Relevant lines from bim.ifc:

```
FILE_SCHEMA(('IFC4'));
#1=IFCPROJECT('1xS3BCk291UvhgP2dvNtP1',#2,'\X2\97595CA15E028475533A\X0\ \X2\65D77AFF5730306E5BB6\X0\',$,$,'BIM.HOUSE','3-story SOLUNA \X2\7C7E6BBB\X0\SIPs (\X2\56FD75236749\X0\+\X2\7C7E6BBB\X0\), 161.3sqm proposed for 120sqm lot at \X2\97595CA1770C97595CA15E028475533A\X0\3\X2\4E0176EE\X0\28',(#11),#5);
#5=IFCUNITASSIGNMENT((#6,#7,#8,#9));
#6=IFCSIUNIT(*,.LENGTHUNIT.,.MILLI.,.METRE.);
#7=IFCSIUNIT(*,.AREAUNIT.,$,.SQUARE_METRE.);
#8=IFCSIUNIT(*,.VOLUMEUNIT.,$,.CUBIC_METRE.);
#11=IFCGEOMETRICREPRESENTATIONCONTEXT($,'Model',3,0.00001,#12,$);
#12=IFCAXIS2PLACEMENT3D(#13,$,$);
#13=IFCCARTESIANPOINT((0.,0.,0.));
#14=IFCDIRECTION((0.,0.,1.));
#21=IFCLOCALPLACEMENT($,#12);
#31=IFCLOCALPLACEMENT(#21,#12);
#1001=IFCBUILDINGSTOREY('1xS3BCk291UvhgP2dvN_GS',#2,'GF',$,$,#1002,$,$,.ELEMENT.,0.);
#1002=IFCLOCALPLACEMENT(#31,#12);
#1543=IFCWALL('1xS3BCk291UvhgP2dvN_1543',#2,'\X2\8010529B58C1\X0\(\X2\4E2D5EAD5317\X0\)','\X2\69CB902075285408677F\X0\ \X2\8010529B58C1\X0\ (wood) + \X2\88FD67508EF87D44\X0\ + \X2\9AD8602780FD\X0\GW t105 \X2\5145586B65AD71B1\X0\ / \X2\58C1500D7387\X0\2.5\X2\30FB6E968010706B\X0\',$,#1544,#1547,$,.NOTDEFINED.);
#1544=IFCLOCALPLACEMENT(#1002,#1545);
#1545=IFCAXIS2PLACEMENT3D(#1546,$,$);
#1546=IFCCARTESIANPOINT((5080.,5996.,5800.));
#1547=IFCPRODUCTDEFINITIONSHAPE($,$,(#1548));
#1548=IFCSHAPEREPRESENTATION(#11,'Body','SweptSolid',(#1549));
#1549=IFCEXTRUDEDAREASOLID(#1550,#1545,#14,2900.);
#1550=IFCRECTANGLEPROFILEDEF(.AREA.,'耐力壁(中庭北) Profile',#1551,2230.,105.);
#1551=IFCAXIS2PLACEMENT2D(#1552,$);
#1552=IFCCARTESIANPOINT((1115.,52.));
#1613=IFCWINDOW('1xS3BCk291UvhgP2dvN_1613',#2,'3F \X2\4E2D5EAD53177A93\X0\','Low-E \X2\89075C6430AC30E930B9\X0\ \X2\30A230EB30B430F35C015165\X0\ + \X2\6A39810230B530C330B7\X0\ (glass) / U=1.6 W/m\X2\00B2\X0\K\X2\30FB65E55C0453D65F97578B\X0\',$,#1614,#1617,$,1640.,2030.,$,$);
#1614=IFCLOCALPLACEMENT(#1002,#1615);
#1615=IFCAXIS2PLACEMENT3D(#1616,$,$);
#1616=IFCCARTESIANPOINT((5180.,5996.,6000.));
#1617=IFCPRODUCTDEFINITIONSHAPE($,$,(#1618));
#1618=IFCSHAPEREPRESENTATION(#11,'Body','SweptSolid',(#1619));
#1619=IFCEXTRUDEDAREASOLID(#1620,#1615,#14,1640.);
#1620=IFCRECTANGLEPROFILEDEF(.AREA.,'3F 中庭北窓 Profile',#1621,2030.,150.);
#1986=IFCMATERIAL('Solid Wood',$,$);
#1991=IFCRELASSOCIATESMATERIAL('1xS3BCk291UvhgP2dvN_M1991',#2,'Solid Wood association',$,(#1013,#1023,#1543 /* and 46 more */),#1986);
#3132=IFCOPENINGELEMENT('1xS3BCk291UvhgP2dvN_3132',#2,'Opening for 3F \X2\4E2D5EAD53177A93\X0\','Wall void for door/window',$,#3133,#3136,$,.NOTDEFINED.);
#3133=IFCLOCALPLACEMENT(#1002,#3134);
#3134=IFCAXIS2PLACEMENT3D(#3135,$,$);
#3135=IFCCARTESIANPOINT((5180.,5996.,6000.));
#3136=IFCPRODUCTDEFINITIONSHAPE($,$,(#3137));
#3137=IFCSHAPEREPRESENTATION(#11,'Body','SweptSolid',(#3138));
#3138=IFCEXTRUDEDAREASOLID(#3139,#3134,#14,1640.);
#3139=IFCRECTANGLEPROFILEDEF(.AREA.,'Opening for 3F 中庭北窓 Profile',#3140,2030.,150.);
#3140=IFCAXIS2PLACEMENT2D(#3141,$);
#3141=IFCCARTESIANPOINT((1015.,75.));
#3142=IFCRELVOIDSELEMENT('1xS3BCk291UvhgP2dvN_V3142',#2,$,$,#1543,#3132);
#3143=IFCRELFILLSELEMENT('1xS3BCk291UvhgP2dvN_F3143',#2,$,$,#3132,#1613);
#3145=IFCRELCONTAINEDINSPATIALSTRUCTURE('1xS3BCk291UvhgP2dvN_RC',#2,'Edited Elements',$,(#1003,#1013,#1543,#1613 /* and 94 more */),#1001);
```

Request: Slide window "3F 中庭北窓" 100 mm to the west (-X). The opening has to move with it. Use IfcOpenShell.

```python
import ifcopenshell
import ifcopenshell.api.geometry
import ifcopenshell.util.placement
import ifcopenshell.util.unit

model = ifcopenshell.open("bim.ifc")
unit_scale = ifcopenshell.util.unit.calculate_unit_scale(model)

window = model.by_guid("1xS3BCk291UvhgP2dvN_1613")
opening = window.FillsVoids[0].RelatingOpeningElement
wall = opening.VoidsElements[0].RelatingBuildingElement

wall_matrix = ifcopenshell.util.placement.get_local_placement(wall.ObjectPlacement)
shift = wall_matrix[:3, 0] * -0.1 / unit_scale
before = ifcopenshell.util.placement.get_local_placement(window.ObjectPlacement)[:3, 3].copy()

# The window is not placed relative to its opening, so move both.
for product in (opening, window):
    matrix = ifcopenshell.util.placement.get_local_placement(product.ObjectPlacement)
    matrix[:3, 3] += shift
    ifcopenshell.api.geometry.edit_object_placement(model, product=product, matrix=matrix, is_si=False)

after = ifcopenshell.util.placement.get_local_placement(window.ObjectPlacement)[:3, 3]
print("window moved by", (after - before).round(3) + 0.0)

model.write("bim_updated.ifc")
```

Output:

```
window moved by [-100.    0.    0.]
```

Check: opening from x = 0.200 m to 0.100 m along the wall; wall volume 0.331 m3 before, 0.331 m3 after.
